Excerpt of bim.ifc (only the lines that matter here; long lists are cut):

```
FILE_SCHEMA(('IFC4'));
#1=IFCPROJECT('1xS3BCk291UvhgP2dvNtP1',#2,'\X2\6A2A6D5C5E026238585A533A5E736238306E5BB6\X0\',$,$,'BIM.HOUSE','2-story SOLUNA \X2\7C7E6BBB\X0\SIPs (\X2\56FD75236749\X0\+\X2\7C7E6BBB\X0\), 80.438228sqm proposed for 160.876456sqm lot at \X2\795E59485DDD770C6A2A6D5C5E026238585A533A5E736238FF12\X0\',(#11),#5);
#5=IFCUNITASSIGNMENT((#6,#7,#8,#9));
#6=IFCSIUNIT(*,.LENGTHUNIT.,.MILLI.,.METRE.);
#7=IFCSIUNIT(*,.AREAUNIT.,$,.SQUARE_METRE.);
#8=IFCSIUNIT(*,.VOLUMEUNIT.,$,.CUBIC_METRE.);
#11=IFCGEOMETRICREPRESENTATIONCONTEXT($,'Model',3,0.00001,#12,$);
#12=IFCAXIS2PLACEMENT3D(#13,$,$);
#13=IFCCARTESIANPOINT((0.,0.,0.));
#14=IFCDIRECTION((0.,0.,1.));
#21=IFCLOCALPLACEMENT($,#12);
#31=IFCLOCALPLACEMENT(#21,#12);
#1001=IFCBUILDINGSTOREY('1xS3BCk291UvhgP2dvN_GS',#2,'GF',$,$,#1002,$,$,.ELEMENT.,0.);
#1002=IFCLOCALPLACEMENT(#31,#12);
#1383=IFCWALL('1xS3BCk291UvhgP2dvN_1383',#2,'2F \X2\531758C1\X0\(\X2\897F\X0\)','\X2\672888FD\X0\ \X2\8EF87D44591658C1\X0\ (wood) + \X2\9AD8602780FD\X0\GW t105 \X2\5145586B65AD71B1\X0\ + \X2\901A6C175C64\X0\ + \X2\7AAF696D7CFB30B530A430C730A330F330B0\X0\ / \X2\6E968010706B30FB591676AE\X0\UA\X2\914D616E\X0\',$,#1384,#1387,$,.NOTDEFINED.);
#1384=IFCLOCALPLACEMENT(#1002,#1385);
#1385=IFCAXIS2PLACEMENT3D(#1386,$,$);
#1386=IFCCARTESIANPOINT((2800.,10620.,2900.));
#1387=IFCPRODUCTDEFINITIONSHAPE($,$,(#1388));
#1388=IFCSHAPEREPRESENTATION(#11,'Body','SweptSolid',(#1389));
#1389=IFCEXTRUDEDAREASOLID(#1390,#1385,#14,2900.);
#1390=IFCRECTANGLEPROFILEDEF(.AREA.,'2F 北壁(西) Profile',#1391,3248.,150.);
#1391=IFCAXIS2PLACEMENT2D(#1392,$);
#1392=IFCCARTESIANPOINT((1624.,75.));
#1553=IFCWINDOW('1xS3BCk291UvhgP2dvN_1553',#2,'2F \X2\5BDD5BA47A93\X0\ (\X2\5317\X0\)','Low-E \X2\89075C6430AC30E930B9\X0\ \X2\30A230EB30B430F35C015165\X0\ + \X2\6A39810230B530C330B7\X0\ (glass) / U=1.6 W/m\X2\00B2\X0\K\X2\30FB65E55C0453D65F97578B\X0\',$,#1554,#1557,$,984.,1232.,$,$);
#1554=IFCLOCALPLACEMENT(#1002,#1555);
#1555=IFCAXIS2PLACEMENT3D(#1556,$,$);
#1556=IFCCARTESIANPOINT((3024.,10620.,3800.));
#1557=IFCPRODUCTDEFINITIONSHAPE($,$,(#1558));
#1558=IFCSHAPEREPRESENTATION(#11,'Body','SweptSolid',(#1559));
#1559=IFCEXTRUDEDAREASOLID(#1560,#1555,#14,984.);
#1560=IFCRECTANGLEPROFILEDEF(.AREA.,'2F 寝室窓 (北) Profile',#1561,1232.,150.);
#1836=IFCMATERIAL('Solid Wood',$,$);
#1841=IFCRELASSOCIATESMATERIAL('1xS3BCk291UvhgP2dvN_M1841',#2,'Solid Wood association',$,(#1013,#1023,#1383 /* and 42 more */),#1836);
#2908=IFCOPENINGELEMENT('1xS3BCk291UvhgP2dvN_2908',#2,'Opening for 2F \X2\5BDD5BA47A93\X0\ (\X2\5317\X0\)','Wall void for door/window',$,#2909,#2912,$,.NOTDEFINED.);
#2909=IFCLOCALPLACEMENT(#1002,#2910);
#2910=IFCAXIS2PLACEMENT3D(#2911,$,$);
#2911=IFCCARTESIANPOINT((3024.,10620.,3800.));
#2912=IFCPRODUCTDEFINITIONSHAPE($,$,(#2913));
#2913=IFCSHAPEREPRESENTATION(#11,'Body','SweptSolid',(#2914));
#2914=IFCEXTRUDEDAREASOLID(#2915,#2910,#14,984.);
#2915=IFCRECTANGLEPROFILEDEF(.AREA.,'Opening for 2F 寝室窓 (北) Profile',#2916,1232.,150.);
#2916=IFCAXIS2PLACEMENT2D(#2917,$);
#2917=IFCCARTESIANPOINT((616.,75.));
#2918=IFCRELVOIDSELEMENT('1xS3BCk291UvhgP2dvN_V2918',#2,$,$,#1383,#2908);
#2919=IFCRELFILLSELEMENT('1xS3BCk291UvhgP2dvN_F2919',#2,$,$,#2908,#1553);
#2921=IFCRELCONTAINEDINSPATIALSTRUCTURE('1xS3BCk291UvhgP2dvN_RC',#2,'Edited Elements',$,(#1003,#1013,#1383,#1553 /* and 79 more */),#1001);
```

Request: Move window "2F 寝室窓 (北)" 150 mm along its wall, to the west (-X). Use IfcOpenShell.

```python
import ifcopenshell
import ifcopenshell.api.geometry
import ifcopenshell.util.placement
import ifcopenshell.util.unit

model = ifcopenshell.open("bim.ifc")
unit_scale = ifcopenshell.util.unit.calculate_unit_scale(model)

window = model.by_id(1553)
opening = window.FillsVoids[0].RelatingOpeningElement
wall = opening.VoidsElements[0].RelatingBuildingElement

wall_matrix = ifcopenshell.util.placement.get_local_placement(wall.ObjectPlacement)
shift = wall_matrix[:3, 0] * -0.15 / unit_scale
before = ifcopenshell.util.placement.get_local_placement(window.ObjectPlacement)[:3, 3].copy()

# The window is not placed relative to its opening, so move both.
for product in (opening, window):
    matrix = ifcopenshell.util.placement.get_local_placement(product.ObjectPlacement)
    matrix[:3, 3] += shift
    ifcopenshell.api.geometry.edit_object_placement(model, product=product, matrix=matrix, is_si=False)

after = ifcopenshell.util.placement.get_local_placement(window.ObjectPlacement)[:3, 3]
print("window moved by", (after - before).round(3) + 0.0)

model.write("bim_edited.ifc")
```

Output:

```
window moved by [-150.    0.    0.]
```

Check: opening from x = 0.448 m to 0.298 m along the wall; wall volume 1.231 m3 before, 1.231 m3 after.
